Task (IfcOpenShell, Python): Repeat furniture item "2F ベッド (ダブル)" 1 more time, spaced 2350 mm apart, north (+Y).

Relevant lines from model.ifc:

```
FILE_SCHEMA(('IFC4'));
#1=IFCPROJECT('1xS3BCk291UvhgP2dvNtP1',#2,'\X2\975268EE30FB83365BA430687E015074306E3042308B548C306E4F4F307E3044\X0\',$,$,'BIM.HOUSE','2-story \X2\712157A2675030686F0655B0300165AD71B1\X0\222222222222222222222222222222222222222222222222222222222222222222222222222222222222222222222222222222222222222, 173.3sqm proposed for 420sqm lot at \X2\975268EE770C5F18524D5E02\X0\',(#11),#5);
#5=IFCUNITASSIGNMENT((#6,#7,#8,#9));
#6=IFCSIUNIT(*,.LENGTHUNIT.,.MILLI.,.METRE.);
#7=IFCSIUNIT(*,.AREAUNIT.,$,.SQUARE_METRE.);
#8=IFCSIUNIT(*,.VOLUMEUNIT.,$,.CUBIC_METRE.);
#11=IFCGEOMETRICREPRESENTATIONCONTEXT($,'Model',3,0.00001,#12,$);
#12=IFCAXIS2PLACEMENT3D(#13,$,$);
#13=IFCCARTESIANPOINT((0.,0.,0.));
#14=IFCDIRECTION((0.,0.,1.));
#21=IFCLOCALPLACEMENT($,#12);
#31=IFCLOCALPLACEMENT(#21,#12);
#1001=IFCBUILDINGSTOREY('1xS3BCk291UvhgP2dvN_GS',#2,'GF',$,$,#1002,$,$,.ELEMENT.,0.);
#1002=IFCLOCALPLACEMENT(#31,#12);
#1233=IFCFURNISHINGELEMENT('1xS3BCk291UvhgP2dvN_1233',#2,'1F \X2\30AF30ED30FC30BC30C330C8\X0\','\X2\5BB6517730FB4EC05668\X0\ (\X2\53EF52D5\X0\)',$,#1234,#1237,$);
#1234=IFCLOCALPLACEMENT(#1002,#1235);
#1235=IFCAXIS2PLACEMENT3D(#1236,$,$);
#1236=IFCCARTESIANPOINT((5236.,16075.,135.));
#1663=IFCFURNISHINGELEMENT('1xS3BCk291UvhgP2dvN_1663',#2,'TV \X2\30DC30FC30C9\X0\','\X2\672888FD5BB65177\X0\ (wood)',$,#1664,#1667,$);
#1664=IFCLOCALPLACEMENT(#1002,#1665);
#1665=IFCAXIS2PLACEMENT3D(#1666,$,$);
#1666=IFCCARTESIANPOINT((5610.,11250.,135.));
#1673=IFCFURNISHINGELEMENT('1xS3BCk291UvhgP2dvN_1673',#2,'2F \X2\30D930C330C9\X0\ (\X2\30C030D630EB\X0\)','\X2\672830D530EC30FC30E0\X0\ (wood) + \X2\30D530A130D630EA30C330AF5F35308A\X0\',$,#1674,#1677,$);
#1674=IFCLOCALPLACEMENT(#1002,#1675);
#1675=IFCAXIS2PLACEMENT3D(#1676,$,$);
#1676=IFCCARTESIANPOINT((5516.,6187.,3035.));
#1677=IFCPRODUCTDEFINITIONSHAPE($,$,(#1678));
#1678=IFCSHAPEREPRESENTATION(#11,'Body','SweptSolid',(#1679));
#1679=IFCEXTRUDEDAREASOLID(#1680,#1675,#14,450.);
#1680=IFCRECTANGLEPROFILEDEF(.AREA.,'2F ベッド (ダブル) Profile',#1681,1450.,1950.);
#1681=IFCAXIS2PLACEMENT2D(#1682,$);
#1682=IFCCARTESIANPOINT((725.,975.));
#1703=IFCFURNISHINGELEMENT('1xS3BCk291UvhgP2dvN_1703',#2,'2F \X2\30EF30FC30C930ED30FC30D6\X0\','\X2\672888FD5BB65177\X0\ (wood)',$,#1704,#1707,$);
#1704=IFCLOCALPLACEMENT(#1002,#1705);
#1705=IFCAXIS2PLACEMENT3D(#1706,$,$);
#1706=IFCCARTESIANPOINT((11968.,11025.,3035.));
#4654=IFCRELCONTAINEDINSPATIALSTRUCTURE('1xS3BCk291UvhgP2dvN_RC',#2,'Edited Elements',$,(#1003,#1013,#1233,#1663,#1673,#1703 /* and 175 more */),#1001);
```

```python
import numpy as np
import ifcopenshell
import ifcopenshell.api.geometry
import ifcopenshell.api.root
import ifcopenshell.util.element
import ifcopenshell.util.placement
import ifcopenshell.util.unit

model = ifcopenshell.open("model.ifc")
unit_scale = ifcopenshell.util.unit.calculate_unit_scale(model)


def reuse_history(source, copy):
    """copy_class also copies each property set's owner history, people and application; keep the originals."""
    for rel in copy.IsDefinedBy:
        if rel.is_a("IfcRelDefinesByProperties") and (history := rel.RelatingPropertyDefinition.OwnerHistory):
            rel.RelatingPropertyDefinition.OwnerHistory = source.OwnerHistory
            ifcopenshell.util.element.remove_deep2(model, history)


source = model.by_guid("1xS3BCk291UvhgP2dvN_1673")
base = ifcopenshell.util.placement.get_local_placement(source.ObjectPlacement)
step = np.array([0.0, 1.0, 0.0]) * 2.35 / unit_scale

for i in range(1, 2):
    copy = ifcopenshell.api.root.copy_class(model, product=source)
    copy.Representation = ifcopenshell.util.element.copy_deep(
        model, source.Representation, exclude=["IfcGeometricRepresentationContext", "IfcRepresentationMap"]
    )
    reuse_history(source, copy)
    matrix = base.copy()
    matrix[:3, 3] += i * step
    print("added at", matrix[:3, 3].round(3) + 0.0)
    ifcopenshell.api.geometry.edit_object_placement(model, product=copy, matrix=matrix, is_si=False)

model.write("model_edited.ifc")
```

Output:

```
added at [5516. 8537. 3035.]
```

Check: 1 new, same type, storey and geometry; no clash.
